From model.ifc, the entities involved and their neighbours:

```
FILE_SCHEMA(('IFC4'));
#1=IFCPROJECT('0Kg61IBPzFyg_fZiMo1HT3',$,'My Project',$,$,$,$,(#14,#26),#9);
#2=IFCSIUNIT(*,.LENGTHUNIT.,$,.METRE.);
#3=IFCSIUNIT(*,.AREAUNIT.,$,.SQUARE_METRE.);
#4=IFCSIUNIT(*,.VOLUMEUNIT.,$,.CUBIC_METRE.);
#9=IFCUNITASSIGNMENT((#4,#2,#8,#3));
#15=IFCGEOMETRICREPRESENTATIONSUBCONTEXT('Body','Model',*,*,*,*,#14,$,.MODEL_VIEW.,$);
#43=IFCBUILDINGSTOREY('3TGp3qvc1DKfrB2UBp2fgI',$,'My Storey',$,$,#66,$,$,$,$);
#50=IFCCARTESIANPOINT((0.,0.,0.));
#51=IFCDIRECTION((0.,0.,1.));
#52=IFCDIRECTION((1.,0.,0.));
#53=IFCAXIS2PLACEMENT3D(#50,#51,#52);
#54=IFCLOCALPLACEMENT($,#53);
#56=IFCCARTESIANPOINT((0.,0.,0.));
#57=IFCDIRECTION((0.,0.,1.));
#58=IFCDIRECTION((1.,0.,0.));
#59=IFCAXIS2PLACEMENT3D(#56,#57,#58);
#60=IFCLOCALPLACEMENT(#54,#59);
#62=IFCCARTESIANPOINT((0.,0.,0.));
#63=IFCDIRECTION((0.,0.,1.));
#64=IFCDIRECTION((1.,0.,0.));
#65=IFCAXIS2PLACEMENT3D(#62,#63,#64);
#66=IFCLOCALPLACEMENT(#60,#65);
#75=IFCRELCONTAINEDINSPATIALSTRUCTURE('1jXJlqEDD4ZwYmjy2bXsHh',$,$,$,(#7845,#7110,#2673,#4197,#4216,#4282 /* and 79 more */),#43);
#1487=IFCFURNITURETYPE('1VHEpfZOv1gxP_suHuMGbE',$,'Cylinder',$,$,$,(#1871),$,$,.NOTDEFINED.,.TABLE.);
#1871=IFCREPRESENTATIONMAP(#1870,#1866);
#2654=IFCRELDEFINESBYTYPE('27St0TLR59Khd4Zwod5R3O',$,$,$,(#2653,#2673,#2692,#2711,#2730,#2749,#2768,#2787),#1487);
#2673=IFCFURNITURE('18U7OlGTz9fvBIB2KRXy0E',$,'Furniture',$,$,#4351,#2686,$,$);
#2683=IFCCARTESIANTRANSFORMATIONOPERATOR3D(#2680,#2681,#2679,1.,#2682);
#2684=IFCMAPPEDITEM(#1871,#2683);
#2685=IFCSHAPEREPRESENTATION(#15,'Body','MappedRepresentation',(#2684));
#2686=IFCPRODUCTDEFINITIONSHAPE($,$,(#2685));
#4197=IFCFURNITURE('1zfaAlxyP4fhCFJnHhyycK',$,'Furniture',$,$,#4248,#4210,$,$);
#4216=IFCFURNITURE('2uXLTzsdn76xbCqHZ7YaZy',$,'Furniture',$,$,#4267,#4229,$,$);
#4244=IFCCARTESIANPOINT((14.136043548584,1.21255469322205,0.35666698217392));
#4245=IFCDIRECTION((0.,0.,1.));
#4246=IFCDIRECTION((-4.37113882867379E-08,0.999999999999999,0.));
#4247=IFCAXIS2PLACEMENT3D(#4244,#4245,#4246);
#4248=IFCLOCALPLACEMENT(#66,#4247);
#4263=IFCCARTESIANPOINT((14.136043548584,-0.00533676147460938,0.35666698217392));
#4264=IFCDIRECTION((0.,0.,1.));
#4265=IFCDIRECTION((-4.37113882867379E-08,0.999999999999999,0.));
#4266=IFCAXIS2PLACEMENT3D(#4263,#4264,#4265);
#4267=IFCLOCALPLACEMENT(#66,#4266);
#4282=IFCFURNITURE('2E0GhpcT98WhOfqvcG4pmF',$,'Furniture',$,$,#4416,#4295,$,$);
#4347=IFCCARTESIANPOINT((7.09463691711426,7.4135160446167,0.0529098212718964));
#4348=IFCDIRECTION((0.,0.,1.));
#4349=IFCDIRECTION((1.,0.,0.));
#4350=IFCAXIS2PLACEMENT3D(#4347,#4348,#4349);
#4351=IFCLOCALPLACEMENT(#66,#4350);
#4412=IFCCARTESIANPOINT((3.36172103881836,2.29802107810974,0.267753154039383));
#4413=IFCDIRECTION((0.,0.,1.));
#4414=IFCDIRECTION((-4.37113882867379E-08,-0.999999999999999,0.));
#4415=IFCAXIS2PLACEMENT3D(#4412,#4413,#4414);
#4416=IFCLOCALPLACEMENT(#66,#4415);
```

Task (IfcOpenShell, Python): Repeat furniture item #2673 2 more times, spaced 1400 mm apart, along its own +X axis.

```python
import ifcopenshell
import ifcopenshell.api.geometry
import ifcopenshell.api.root
import ifcopenshell.util.element
import ifcopenshell.util.placement

model = ifcopenshell.open("model.ifc")

source = model.by_id(2673)
base = ifcopenshell.util.placement.get_local_placement(source.ObjectPlacement)
step = base[:3, 0] * 1.4

for i in range(1, 3):
    copy = ifcopenshell.api.root.copy_class(model, product=source)
    copy.Representation = ifcopenshell.util.element.copy_deep(
        model, source.Representation, exclude=["IfcGeometricRepresentationContext", "IfcRepresentationMap"]
    )
    matrix = base.copy()
    matrix[:3, 3] += i * step
    print("added at", matrix[:3, 3].round(3) + 0.0)
    ifcopenshell.api.geometry.edit_object_placement(model, product=copy, matrix=matrix, is_si=False)

model.write("model_edited.ifc")
```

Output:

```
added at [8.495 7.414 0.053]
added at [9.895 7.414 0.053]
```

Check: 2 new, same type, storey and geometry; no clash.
